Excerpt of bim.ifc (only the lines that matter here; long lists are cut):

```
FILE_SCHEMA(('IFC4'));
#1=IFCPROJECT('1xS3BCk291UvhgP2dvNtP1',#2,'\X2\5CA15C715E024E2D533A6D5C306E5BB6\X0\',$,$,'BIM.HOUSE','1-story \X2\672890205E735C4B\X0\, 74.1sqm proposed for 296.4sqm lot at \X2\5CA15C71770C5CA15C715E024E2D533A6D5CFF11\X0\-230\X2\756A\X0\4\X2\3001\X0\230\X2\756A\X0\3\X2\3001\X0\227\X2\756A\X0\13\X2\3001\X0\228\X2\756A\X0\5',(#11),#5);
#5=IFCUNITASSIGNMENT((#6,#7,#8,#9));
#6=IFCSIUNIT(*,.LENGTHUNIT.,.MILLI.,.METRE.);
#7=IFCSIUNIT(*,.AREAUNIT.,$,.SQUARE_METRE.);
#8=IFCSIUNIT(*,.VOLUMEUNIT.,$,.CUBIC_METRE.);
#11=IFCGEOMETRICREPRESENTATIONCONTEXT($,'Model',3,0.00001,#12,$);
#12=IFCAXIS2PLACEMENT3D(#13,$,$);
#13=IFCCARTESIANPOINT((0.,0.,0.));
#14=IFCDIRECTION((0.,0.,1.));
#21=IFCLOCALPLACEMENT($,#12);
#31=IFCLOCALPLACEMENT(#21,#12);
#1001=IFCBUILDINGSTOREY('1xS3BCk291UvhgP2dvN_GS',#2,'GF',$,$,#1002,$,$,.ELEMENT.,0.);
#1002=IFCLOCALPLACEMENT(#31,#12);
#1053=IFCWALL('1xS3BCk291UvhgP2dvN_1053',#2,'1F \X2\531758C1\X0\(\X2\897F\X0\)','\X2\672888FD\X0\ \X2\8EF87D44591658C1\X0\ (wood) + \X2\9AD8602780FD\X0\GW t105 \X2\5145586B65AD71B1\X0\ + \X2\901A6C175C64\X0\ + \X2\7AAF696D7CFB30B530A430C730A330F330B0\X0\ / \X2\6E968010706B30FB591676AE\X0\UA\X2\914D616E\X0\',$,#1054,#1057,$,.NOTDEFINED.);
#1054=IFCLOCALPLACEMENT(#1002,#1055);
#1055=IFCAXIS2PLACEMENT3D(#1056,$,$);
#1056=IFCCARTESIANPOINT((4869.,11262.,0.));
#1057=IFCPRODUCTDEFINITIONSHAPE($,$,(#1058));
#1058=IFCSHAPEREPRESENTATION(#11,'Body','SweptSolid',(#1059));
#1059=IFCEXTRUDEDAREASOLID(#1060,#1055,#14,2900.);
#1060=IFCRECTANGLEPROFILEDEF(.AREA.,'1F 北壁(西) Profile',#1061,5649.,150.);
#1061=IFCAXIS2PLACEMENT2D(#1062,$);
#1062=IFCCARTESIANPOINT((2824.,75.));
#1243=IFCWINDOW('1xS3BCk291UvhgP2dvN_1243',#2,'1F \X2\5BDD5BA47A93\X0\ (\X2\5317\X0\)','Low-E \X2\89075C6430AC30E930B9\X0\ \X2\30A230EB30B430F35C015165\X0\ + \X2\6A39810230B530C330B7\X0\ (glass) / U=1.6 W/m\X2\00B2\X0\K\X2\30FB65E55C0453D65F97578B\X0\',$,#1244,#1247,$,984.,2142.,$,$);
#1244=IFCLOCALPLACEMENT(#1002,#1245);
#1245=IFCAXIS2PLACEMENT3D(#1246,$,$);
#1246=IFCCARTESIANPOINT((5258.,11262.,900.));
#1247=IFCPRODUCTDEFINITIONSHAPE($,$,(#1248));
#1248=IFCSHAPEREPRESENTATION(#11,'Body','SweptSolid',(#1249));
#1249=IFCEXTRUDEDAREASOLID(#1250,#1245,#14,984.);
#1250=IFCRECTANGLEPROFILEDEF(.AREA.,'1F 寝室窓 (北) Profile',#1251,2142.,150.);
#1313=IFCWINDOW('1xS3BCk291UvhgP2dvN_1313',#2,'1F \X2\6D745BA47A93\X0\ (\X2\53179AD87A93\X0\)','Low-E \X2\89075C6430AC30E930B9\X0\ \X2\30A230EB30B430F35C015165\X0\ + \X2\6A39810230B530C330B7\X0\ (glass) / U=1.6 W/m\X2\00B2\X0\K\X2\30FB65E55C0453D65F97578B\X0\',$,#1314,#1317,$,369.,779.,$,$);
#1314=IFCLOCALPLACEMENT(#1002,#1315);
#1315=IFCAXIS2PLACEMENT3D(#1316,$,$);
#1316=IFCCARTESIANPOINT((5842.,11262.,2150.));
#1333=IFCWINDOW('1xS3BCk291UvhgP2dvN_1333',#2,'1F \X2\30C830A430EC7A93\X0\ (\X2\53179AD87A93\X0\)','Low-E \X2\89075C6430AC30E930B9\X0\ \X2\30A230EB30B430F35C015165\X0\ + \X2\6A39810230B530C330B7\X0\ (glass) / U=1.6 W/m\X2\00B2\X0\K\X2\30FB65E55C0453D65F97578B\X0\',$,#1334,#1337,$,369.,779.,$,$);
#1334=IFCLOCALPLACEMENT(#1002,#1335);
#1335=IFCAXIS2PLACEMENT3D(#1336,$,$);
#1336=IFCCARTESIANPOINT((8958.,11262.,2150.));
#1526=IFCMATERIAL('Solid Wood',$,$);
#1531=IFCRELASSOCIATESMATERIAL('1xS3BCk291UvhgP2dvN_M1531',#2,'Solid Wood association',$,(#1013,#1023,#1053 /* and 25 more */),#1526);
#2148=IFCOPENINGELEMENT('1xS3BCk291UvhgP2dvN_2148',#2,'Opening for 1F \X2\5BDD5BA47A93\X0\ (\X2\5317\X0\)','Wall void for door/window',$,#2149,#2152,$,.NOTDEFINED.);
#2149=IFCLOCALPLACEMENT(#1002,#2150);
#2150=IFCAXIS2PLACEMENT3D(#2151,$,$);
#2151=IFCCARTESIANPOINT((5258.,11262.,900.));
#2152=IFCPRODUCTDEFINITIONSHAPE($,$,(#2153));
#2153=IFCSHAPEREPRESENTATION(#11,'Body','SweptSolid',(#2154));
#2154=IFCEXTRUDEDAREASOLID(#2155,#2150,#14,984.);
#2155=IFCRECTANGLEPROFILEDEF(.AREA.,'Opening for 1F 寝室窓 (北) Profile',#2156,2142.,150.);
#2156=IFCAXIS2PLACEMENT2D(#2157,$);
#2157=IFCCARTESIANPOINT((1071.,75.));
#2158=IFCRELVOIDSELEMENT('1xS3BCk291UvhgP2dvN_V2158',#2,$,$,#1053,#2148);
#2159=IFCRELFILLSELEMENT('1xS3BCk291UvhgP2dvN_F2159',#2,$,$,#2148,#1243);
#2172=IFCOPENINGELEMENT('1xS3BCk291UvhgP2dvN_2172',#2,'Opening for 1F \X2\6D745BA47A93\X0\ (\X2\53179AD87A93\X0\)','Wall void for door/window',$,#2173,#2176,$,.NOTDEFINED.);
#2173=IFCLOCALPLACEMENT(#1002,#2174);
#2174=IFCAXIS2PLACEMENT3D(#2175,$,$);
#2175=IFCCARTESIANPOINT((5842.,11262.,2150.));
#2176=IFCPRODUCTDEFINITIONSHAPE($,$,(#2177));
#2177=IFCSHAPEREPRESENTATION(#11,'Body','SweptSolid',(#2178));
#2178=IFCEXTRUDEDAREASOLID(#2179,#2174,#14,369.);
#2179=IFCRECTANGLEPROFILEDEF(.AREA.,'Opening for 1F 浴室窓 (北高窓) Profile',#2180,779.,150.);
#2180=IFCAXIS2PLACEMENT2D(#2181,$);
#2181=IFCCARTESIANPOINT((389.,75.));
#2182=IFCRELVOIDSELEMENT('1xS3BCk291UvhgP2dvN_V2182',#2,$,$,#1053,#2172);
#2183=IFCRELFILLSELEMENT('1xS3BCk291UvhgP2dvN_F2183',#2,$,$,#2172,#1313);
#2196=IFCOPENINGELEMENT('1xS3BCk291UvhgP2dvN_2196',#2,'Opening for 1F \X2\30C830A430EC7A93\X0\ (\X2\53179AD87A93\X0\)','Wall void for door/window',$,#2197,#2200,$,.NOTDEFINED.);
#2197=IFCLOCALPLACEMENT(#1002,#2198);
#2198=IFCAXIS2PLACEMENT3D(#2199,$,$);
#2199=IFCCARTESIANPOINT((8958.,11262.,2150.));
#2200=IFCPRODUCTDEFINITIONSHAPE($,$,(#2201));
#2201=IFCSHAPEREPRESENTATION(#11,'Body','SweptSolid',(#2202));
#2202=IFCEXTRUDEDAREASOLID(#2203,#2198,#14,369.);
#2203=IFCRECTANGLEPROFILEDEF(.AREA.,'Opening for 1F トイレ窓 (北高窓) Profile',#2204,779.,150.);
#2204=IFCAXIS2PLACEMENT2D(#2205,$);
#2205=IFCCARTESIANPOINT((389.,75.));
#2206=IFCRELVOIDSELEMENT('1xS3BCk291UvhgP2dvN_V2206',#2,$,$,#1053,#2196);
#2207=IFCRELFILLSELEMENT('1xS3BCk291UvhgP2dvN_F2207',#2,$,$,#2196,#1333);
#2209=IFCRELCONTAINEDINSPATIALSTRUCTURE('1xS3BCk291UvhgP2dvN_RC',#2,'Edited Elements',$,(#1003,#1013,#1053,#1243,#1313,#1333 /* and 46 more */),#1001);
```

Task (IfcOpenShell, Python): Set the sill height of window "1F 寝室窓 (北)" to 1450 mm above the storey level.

```python
import numpy as np
import ifcopenshell
import ifcopenshell.api.geometry
import ifcopenshell.geom
import ifcopenshell.util.element
import ifcopenshell.util.placement
import ifcopenshell.util.shape
import ifcopenshell.util.unit

model = ifcopenshell.open("bim.ifc")
unit_scale = ifcopenshell.util.unit.calculate_unit_scale(model)

window = model.by_guid("1xS3BCk291UvhgP2dvN_1243")
opening = window.FillsVoids[0].RelatingOpeningElement
storey = ifcopenshell.util.element.get_container(window, ifc_class="IfcBuildingStorey")
level = ifcopenshell.util.placement.get_local_placement(storey.ObjectPlacement)[2, 3]

# The opening's origin need not be at the sill, so measure its lowest point.
shape = ifcopenshell.geom.create_shape(ifcopenshell.geom.settings(), opening)
bottom = ifcopenshell.util.shape.get_shape_bottom_elevation(shape, shape.geometry) / unit_scale
dz = level + 1450.0 - bottom

shift = np.array([0.0, 0.0, dz])
# The window is not placed relative to its opening, so move both.
for product in (opening, window):
    matrix = ifcopenshell.util.placement.get_local_placement(product.ObjectPlacement)
    matrix[:3, 3] += shift
    ifcopenshell.api.geometry.edit_object_placement(model, product=product, matrix=matrix, is_si=False)

print(f"moved by {dz * unit_scale:+.3f} m")

model.write("bim_rev.ifc")
```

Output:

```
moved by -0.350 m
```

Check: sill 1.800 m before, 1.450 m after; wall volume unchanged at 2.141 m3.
